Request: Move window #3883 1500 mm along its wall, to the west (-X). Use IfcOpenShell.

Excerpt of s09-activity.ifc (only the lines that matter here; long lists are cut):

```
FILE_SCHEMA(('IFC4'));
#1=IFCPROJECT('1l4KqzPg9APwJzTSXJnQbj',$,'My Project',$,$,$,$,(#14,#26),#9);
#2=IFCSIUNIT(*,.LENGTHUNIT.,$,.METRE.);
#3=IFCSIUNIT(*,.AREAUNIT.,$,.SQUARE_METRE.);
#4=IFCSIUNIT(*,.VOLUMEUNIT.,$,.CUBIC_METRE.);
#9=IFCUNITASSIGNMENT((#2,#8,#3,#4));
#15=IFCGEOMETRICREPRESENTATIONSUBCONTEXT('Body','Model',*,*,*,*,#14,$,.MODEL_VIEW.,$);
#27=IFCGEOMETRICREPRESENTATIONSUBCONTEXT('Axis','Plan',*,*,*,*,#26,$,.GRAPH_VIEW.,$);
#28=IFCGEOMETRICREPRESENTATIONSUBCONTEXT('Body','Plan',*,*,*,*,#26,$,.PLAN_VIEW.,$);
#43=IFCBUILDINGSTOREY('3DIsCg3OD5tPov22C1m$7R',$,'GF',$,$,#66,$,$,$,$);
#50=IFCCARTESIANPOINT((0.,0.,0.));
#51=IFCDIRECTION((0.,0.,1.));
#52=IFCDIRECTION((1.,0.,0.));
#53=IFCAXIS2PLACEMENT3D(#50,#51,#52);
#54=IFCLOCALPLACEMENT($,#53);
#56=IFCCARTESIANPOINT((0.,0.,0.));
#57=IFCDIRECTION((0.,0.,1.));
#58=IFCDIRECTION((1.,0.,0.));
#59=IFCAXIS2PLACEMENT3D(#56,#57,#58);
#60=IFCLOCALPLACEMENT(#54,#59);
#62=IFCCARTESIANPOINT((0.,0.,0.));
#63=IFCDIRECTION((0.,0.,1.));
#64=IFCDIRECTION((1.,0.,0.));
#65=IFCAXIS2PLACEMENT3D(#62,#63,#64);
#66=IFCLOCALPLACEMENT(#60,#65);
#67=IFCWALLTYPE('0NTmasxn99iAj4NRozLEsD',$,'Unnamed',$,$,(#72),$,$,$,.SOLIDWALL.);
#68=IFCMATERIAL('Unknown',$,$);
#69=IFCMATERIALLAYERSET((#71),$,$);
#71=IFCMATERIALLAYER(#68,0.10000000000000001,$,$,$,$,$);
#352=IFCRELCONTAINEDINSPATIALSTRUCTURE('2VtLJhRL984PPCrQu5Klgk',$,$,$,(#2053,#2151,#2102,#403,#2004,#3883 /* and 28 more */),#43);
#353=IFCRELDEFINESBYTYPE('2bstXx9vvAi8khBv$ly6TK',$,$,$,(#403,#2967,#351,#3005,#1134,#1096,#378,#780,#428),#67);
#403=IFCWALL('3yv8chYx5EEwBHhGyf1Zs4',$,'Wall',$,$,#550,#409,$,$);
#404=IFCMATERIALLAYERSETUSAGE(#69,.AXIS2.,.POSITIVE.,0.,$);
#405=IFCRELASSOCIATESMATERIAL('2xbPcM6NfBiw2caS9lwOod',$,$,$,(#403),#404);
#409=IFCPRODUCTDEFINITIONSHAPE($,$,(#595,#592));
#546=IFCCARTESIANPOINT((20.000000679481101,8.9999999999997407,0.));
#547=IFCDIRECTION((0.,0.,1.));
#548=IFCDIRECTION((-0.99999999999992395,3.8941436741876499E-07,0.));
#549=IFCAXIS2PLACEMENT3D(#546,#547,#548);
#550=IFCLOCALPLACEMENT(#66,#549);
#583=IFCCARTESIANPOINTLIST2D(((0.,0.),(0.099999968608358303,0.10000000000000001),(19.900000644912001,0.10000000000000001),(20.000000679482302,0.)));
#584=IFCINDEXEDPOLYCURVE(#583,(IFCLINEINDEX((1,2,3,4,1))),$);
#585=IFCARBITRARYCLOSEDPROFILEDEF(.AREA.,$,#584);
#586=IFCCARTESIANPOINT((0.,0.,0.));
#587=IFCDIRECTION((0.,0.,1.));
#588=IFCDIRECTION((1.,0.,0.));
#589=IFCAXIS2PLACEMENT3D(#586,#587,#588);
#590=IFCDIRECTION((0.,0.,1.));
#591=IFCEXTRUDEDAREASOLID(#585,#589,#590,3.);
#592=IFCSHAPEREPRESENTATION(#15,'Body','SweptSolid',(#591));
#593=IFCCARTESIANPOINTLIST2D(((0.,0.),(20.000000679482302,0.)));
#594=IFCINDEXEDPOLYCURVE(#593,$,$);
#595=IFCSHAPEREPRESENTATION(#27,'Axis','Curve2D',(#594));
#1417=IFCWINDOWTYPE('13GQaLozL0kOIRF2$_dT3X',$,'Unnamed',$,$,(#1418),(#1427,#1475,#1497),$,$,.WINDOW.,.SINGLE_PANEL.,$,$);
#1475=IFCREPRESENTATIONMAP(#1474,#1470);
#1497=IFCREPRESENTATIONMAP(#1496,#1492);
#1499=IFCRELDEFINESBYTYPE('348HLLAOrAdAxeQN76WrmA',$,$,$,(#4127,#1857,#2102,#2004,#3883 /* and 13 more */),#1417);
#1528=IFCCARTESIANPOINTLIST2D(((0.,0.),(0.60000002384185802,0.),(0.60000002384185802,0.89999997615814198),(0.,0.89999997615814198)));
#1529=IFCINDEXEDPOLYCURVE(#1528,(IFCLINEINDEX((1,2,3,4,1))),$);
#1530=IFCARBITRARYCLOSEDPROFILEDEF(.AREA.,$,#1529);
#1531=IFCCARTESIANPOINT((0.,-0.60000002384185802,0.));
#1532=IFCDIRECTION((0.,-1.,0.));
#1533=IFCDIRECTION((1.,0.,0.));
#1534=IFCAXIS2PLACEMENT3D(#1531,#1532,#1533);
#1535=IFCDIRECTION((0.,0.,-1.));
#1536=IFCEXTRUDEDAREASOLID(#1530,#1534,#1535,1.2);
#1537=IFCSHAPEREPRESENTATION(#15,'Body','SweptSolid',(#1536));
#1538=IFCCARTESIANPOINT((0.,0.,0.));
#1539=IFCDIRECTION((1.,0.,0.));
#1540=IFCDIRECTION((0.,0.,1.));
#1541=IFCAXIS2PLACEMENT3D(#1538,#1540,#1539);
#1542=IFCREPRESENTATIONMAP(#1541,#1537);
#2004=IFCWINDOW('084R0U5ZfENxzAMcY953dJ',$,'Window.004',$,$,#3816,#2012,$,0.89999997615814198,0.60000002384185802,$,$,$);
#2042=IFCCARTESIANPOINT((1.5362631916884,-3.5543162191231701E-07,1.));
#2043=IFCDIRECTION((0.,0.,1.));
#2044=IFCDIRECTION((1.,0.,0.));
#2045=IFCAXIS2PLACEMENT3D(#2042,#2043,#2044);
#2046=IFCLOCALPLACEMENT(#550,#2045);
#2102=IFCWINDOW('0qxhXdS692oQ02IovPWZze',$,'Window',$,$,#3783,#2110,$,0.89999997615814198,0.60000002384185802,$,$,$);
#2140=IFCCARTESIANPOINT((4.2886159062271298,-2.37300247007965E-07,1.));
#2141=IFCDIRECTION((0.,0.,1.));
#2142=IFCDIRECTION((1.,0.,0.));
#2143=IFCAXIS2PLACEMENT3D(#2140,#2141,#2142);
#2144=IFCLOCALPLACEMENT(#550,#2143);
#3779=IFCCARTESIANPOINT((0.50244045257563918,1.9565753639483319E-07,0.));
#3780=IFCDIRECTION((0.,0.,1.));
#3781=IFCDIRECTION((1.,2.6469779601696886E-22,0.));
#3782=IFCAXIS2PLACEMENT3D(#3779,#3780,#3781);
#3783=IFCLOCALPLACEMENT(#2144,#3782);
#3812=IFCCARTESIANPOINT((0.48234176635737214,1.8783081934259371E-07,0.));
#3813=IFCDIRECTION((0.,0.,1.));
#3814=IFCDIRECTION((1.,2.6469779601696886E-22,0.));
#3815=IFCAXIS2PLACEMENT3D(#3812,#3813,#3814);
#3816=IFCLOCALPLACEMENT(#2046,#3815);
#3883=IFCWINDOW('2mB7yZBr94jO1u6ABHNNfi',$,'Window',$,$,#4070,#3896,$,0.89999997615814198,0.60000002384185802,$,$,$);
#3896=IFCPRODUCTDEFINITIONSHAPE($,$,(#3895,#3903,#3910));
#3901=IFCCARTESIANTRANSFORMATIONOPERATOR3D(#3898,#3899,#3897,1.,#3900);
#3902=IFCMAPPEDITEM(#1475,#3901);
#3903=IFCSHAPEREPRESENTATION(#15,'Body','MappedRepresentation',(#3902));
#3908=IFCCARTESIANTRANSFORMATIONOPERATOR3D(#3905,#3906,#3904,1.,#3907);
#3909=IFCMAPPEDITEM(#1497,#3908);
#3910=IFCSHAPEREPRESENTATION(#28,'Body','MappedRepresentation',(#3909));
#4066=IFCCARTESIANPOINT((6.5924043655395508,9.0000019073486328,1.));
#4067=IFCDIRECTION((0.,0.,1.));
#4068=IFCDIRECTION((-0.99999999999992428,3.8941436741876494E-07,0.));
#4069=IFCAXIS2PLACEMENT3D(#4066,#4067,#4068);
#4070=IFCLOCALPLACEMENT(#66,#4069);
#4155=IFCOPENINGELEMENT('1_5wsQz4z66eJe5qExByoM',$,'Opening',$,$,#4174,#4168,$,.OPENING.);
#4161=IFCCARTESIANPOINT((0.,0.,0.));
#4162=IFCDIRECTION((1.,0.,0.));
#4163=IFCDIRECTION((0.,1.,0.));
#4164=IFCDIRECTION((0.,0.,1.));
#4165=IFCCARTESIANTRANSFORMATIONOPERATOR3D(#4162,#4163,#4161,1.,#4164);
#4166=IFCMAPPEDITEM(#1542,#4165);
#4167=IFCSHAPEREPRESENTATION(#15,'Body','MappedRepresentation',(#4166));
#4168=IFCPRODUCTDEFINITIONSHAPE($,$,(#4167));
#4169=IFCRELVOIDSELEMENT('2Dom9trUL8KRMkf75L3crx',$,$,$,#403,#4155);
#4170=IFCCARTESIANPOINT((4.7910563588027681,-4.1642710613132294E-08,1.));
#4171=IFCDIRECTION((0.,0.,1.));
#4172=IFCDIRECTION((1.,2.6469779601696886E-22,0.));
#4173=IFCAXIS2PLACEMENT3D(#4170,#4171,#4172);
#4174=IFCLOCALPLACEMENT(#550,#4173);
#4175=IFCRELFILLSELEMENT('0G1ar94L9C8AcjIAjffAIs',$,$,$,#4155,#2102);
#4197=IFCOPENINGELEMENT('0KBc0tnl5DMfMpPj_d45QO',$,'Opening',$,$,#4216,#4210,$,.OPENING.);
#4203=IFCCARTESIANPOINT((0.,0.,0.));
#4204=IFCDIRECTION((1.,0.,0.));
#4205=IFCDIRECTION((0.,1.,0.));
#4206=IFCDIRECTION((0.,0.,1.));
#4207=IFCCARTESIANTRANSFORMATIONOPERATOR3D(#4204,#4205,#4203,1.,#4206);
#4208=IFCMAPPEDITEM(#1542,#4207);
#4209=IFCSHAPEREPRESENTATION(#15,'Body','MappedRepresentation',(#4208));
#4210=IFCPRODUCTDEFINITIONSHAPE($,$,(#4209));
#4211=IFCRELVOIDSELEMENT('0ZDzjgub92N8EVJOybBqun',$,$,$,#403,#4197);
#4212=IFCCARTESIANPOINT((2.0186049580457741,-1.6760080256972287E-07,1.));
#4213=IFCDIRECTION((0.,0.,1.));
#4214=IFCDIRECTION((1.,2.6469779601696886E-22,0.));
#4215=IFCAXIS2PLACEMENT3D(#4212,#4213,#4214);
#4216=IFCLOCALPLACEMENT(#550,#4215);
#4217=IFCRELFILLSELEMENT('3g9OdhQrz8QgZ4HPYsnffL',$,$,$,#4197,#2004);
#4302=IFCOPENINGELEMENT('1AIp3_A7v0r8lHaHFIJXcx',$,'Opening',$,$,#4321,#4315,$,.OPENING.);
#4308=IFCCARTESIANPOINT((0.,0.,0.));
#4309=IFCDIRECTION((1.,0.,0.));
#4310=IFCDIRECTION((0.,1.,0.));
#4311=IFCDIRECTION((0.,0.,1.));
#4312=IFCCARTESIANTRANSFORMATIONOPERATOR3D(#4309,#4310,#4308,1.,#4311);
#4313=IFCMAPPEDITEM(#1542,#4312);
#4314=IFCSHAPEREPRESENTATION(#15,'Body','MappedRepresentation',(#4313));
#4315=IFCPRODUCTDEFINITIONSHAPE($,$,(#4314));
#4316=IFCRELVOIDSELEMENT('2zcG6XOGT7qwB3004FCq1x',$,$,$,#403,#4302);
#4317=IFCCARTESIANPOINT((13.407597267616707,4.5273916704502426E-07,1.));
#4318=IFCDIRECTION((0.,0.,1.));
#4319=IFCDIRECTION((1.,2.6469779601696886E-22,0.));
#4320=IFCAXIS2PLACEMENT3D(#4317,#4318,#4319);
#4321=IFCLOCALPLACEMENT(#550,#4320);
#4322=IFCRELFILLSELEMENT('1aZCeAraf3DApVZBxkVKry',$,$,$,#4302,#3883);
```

```python
import ifcopenshell
import ifcopenshell.api.geometry
import ifcopenshell.util.placement
import ifcopenshell.util.unit

model = ifcopenshell.open("s09-activity.ifc")
unit_scale = ifcopenshell.util.unit.calculate_unit_scale(model)

window = model.by_guid("2mB7yZBr94jO1u6ABHNNfi")
opening = window.FillsVoids[0].RelatingOpeningElement
wall = opening.VoidsElements[0].RelatingBuildingElement

wall_matrix = ifcopenshell.util.placement.get_local_placement(wall.ObjectPlacement)
shift = wall_matrix[:3, 0] * 1.5 / unit_scale
before = ifcopenshell.util.placement.get_local_placement(window.ObjectPlacement)[:3, 3].copy()

# The window is not placed relative to its opening, so move both.
for product in (opening, window):
    matrix = ifcopenshell.util.placement.get_local_placement(product.ObjectPlacement)
    matrix[:3, 3] += shift
    ifcopenshell.api.geometry.edit_object_placement(model, product=product, matrix=matrix, is_si=False)

after = ifcopenshell.util.placement.get_local_placement(window.ObjectPlacement)[:3, 3]
print("window moved by", (after - before).round(3) + 0.0)

model.write("s09-activity_rev.ifc")
```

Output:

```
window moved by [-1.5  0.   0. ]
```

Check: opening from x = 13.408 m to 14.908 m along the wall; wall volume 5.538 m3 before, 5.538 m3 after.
